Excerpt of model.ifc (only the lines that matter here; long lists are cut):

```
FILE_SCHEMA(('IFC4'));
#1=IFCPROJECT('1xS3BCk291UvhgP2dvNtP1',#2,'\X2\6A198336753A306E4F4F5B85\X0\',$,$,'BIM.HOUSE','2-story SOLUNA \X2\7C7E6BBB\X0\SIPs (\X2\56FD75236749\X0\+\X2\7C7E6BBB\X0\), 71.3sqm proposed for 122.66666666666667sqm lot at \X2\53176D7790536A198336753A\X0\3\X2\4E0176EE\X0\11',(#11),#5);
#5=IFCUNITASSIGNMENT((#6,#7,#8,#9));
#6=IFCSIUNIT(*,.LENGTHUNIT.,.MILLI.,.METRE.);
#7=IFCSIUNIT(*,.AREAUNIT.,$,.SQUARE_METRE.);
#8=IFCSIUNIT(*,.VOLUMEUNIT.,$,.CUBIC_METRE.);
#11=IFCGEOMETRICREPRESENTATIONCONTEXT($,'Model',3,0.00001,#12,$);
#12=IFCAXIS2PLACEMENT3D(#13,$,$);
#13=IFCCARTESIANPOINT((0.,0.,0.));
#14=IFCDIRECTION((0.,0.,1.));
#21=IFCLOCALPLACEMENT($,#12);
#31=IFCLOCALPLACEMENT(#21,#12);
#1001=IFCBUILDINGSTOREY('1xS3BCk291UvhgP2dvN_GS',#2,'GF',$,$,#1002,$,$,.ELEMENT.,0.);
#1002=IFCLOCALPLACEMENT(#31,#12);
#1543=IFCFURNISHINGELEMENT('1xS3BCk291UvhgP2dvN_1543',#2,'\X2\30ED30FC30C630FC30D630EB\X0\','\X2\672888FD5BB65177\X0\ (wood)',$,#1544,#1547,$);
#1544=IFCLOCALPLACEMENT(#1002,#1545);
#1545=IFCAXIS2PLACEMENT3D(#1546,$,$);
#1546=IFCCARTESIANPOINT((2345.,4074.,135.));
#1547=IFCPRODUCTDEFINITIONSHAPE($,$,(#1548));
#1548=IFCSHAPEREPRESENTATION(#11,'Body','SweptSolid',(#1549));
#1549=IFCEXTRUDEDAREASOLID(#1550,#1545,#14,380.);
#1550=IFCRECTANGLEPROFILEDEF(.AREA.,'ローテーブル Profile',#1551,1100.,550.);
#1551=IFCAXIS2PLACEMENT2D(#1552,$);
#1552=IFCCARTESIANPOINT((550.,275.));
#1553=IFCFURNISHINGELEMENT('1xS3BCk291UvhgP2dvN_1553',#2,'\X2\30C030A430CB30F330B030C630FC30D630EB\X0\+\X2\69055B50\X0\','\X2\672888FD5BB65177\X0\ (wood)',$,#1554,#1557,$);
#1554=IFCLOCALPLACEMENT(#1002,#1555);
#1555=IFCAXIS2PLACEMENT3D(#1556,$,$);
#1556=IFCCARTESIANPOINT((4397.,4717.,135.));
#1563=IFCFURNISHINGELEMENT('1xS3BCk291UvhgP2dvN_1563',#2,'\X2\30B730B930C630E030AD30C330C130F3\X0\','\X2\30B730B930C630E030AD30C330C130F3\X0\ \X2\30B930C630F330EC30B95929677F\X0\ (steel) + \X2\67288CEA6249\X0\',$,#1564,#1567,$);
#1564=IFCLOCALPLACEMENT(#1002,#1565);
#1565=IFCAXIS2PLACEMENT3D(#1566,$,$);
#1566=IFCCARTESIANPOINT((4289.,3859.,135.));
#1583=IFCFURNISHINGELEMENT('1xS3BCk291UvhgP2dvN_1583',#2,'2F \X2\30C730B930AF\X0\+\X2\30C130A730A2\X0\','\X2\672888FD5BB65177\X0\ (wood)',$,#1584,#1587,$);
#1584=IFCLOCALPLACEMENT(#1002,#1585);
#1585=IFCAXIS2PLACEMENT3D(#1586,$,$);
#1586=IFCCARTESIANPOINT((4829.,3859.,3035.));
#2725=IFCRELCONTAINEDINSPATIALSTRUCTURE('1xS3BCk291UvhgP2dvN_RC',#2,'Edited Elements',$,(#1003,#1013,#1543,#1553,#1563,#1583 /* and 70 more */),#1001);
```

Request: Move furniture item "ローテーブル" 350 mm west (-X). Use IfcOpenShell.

```python
import ifcopenshell
import ifcopenshell.api.geometry
import ifcopenshell.util.placement
import ifcopenshell.util.unit

model = ifcopenshell.open("model.ifc")
unit_scale = ifcopenshell.util.unit.calculate_unit_scale(model)

item = model.by_id(1543)
matrix = ifcopenshell.util.placement.get_local_placement(item.ObjectPlacement)
matrix[0, 3] -= 0.35 / unit_scale
ifcopenshell.api.geometry.edit_object_placement(model, product=item, matrix=matrix, is_si=False)

print(ifcopenshell.util.placement.get_local_placement(item.ObjectPlacement).round(3) + 0.0)

model.write("model_updated.ifc")
```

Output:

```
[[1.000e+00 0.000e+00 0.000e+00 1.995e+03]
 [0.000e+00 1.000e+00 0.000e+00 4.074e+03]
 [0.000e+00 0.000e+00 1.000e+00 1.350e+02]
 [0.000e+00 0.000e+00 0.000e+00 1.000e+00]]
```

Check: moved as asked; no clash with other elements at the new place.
